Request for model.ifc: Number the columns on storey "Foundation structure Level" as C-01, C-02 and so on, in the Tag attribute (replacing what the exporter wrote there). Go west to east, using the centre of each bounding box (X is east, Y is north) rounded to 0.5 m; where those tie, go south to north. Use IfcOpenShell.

First a look at what the model holds.

```python
import ifcopenshell
import ifcopenshell.util.element
import ifcopenshell.util.placement

model = ifcopenshell.open("model.ifc")
print(model.schema)
storey = next(s for s in model.by_type("IfcBuildingStorey") if s.Name == "Foundation structure Level")
columns = [e for e in ifcopenshell.util.element.get_decomposition(storey) if e.is_a("IfcColumn")]
for e in sorted(columns, key=lambda e: e.id()):
    origin = ifcopenshell.util.placement.get_local_placement(e.ObjectPlacement)[:3, 3]
    print(e.id(), e.Tag, e.Name, origin.round(2) + 0.0, sep=" | ")
```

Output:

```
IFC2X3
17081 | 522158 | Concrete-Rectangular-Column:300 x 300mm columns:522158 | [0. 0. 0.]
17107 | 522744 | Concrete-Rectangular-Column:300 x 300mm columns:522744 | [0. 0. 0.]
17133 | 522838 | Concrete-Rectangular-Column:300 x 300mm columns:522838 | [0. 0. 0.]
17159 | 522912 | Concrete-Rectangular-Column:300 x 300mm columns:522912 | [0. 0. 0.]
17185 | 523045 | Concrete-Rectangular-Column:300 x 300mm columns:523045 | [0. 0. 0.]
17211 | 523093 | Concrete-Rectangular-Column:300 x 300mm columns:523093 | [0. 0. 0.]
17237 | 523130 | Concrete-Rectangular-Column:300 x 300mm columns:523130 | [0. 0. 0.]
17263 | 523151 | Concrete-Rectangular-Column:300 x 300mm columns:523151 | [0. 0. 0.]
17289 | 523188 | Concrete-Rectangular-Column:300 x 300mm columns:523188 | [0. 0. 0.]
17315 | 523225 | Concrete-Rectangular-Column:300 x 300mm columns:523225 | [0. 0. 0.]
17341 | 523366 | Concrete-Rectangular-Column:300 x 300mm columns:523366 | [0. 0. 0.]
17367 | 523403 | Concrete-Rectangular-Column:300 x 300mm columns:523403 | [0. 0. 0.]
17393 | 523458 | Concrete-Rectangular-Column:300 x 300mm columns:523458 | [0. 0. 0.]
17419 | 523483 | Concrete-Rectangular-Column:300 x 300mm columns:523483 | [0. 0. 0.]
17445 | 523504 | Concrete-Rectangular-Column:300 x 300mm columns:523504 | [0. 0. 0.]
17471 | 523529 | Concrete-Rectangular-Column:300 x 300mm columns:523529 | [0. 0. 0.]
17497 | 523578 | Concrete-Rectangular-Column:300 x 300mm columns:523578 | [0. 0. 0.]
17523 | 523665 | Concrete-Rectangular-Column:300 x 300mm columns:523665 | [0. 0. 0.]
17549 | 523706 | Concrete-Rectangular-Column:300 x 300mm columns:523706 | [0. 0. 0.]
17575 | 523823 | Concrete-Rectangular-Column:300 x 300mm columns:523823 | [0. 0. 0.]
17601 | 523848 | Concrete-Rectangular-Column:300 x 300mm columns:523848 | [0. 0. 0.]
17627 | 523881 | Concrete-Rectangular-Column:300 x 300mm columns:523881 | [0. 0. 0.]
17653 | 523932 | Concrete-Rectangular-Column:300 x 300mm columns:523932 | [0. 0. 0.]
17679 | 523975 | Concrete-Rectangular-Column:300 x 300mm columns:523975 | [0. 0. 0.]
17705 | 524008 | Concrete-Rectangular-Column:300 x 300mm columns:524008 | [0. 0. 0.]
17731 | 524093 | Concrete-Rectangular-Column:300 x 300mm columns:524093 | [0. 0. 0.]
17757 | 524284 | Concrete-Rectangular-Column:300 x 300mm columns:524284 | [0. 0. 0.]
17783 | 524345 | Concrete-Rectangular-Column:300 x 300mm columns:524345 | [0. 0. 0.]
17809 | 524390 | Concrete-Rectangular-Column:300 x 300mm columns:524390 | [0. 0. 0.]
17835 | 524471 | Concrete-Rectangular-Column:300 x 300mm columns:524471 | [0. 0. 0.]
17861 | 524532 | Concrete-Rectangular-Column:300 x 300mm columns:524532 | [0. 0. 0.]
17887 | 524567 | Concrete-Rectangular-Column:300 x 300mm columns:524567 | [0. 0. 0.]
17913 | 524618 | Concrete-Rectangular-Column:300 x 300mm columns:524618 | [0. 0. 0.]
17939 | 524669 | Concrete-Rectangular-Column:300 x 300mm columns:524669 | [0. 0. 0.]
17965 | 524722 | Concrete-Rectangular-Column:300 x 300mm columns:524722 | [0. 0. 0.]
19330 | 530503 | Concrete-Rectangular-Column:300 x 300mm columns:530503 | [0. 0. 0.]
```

```python
import ifcopenshell
import ifcopenshell.geom
import ifcopenshell.util.element
import ifcopenshell.util.shape

model = ifcopenshell.open("model.ifc")
settings = ifcopenshell.geom.settings()
settings.set("use-world-coords", True)


def centre(element):
    shape = ifcopenshell.geom.create_shape(settings, element)
    return ifcopenshell.util.shape.get_bbox_centroid(shape.geometry)


storey = next(s for s in model.by_type("IfcBuildingStorey") if s.Name == "Foundation structure Level")
columns = [e for e in ifcopenshell.util.element.get_decomposition(storey) if e.is_a("IfcColumn")]

# Insertion points can sit at a corner or the storey origin, so sort by the geometry (in metres).
centres = {e: centre(e) for e in columns}
columns.sort(key=lambda e: (round(centres[e][0] / 0.5), centres[e][1]))

for i, e in enumerate(columns, start=1):
    number = f"C-{i:02d}"
    e.Tag = number
    print(e.id(), number)

model.write("model_v2.ifc")
```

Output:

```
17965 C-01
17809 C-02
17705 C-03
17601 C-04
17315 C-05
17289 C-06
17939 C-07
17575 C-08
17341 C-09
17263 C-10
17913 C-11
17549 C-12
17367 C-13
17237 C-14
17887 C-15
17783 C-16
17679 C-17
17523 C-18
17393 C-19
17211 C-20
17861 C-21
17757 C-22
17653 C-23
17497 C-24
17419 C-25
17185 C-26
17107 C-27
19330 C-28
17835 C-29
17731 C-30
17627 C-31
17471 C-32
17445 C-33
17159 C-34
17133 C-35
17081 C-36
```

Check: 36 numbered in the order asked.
